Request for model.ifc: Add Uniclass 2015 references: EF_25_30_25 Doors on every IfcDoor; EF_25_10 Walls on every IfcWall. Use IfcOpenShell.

First a look at what the model holds.

```python
import ifcopenshell

model = ifcopenshell.open("model.ifc")
print(model.schema)
print("classifications:", [c.Name for c in model.by_type("IfcClassification")])
for ifc_class in ("IfcDoor", "IfcRoof", "IfcStair", "IfcWall", "IfcWindow"):
    print(ifc_class, len(model.by_type(ifc_class)))
```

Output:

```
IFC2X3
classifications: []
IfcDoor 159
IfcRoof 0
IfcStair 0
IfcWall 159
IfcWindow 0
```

```python
import ifcopenshell
import ifcopenshell.api.classification

model = ifcopenshell.open("model.ifc")

# IFC2X3 requires Source and Edition and has no link from the project to the system.
system = model.create_entity("IfcClassification", Source="NBS", Edition="2015", Name="Uniclass 2015")

codes = {
    "IfcDoor": ("EF_25_30_25", "Doors"),
    "IfcWall": ("EF_25_10", "Walls"),
}
for ifc_class, (code, name) in codes.items():
    products = model.by_type(ifc_class)
    ifcopenshell.api.classification.add_reference(
        model, products=products, classification=system, identification=code, name=name
    )
    print(code, len(products))

model.write("model_updated.ifc")
```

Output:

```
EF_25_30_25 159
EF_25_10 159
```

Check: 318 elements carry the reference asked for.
